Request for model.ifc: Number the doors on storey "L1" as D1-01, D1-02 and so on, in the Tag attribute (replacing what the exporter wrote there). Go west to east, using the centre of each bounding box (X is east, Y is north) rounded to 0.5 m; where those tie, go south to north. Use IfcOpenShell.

First a look at what the model holds.

```python
import ifcopenshell
import ifcopenshell.util.element
import ifcopenshell.util.placement

model = ifcopenshell.open("model.ifc")
print(model.schema)
storey = next(s for s in model.by_type("IfcBuildingStorey") if s.Name == "L1")
doors = [e for e in ifcopenshell.util.element.get_decomposition(storey) if e.is_a("IfcDoor")]
for e in sorted(doors, key=lambda e: e.id()):
    origin = ifcopenshell.util.placement.get_local_placement(e.ObjectPlacement)[:3, 3]
    print(e.id(), e.Tag, e.Name, origin.round(2) + 0.0, sep=" | ")
```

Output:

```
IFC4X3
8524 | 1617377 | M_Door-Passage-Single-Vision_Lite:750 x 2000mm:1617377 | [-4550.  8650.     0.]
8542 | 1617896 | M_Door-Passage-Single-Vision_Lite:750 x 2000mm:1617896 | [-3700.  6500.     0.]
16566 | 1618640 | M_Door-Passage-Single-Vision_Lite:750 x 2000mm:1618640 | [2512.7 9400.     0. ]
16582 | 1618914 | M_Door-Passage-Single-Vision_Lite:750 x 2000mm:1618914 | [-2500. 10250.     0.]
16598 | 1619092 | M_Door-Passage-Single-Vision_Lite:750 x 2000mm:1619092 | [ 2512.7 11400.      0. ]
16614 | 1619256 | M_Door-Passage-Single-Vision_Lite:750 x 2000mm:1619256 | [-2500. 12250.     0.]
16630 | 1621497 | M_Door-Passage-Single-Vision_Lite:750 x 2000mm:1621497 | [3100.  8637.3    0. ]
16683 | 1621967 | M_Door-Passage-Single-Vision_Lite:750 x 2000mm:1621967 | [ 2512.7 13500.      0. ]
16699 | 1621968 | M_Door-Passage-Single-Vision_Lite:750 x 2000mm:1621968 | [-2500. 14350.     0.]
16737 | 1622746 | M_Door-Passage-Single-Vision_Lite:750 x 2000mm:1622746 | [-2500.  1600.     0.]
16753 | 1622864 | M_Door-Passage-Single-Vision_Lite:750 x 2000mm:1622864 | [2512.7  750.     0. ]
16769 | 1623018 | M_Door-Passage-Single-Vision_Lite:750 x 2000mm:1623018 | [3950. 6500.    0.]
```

```python
import ifcopenshell
import ifcopenshell.geom
import ifcopenshell.util.element
import ifcopenshell.util.shape

model = ifcopenshell.open("model.ifc")
settings = ifcopenshell.geom.settings()
settings.set("use-world-coords", True)


def centre(element):
    shape = ifcopenshell.geom.create_shape(settings, element)
    return ifcopenshell.util.shape.get_bbox_centroid(shape.geometry)


storey = next(s for s in model.by_type("IfcBuildingStorey") if s.Name == "L1")
doors = [e for e in ifcopenshell.util.element.get_decomposition(storey) if e.is_a("IfcDoor")]

# Insertion points can sit at a corner or the storey origin, so sort by the geometry (in metres).
centres = {e: centre(e) for e in doors}
doors.sort(key=lambda e: (round(centres[e][0] / 0.5), centres[e][1]))

for i, e in enumerate(doors, start=1):
    number = f"D1-{i:02d}"
    e.Tag = number
    print(e.id(), number)

model.write("model-out.ifc")
```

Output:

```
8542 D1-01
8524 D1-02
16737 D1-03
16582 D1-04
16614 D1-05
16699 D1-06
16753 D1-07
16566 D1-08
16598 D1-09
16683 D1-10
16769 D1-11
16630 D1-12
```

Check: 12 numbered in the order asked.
